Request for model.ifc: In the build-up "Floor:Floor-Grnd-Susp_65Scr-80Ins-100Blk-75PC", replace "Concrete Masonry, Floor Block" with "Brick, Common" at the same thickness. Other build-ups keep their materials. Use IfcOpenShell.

First a look at what the model holds.

```python
import ifcopenshell
import ifcopenshell.util.element

model = ifcopenshell.open("model.ifc")
print(model.schema)
for layer_set in model.by_type("IfcMaterialLayerSet"):
    if layer_set.LayerSetName == "Floor:Floor-Grnd-Susp_65Scr-80Ins-100Blk-75PC":
        for layer in layer_set.MaterialLayers:
            print(layer.id(), layer.Material and layer.Material.Name, layer.LayerThickness, sep=" | ")
        print(len(ifcopenshell.util.element.get_elements_by_material(model, layer_set)), "elements and types use it")
print(sorted(m.Name for m in model.by_type("IfcMaterial") if m.Name)[:60])
```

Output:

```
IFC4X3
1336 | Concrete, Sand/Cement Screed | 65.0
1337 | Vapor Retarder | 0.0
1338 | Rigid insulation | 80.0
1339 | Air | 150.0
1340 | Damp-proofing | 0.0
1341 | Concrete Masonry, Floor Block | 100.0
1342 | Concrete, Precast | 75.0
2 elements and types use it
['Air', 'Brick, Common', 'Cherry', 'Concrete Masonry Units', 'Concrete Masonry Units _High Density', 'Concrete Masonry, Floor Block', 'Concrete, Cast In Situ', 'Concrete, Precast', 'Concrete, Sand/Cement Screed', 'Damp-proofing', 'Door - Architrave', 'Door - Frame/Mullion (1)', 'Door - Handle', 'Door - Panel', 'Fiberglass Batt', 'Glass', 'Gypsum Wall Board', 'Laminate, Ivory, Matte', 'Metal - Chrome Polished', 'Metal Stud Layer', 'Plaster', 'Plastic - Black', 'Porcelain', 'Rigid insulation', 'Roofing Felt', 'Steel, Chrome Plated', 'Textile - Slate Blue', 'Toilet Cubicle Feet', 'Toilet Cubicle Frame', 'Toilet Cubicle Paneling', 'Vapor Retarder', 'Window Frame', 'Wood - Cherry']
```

```python
import ifcopenshell
import ifcopenshell.api.material

model = ifcopenshell.open("model.ifc")

layer_set = next(s for s in model.by_type("IfcMaterialLayerSet") if s.LayerSetName == "Floor:Floor-Grnd-Susp_65Scr-80Ins-100Blk-75PC")
layer = next(l for l in layer_set.MaterialLayers if l.Material and l.Material.Name == "Concrete Masonry, Floor Block")
material = next(m for m in model.by_type("IfcMaterial") if m.Name == "Brick, Common")

# Point this one layer at the other material; renaming the old one would change it everywhere.
ifcopenshell.api.material.edit_layer(model, layer=layer, attributes={"Name": material.Name}, material=material)

print([l.Material.Name if l.Material else None for l in layer_set.MaterialLayers])

model.write("model_v2.ifc")
```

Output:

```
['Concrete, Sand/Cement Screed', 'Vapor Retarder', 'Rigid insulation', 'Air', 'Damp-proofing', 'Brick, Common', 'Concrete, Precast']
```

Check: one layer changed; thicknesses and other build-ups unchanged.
